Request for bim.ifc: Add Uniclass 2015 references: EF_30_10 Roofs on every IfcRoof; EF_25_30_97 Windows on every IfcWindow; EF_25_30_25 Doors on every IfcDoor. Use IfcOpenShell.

First a look at what the model holds.

```python
import ifcopenshell

model = ifcopenshell.open("bim.ifc")
print(model.schema)
print("classifications:", [c.Name for c in model.by_type("IfcClassification")])
for ifc_class in ("IfcDoor", "IfcRoof", "IfcStair", "IfcWall", "IfcWindow"):
    print(ifc_class, len(model.by_type(ifc_class)))
```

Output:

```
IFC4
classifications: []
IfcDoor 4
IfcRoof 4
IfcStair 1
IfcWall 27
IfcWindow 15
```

```python
import ifcopenshell
import ifcopenshell.api.classification

model = ifcopenshell.open("bim.ifc")

system = ifcopenshell.api.classification.add_classification(model, classification="Uniclass 2015")

codes = {
    "IfcRoof": ("EF_30_10", "Roofs"),
    "IfcWindow": ("EF_25_30_97", "Windows"),
    "IfcDoor": ("EF_25_30_25", "Doors"),
}
for ifc_class, (code, name) in codes.items():
    products = model.by_type(ifc_class)
    ifcopenshell.api.classification.add_reference(
        model, products=products, classification=system, identification=code, name=name
    )
    print(code, len(products))

model.write("bim_v2.ifc")
```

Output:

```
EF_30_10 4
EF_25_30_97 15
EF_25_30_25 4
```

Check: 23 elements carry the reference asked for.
